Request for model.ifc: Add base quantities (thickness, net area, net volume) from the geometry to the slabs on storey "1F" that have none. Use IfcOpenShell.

First a look at what the model holds.

```python
import ifcopenshell
import ifcopenshell.util.element
import ifcopenshell.util.unit

model = ifcopenshell.open("model.ifc")
print(model.schema)
for unit_type in ("LENGTHUNIT", "AREAUNIT", "VOLUMEUNIT"):
    print(unit_type, ifcopenshell.util.unit.calculate_unit_scale(model, unit_type))
storey = next(s for s in model.by_type("IfcBuildingStorey") if s.Name == "1F")
slabs = [e for e in ifcopenshell.util.element.get_decomposition(storey) if e.is_a("IfcSlab")]
for e in sorted(slabs, key=lambda e: e.id()):
    print(e.id(), e.is_a(), e.Name, list(ifcopenshell.util.element.get_psets(e, qtos_only=True)), sep=" | ")
```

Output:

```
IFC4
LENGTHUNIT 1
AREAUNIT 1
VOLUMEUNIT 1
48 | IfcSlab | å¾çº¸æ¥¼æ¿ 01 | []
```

```python
import ifcopenshell
import ifcopenshell.api.pset
import ifcopenshell.geom
import ifcopenshell.util.element
import ifcopenshell.util.shape
import ifcopenshell.util.unit

model = ifcopenshell.open("model.ifc")
unit_scale = ifcopenshell.util.unit.calculate_unit_scale(model)
area_scale = ifcopenshell.util.unit.calculate_unit_scale(model, "AREAUNIT")
volume_scale = ifcopenshell.util.unit.calculate_unit_scale(model, "VOLUMEUNIT")
settings = ifcopenshell.geom.settings()

storey = next(s for s in model.by_type("IfcBuildingStorey") if s.Name == "1F")
slabs = [e for e in ifcopenshell.util.element.get_decomposition(storey) if e.is_a("IfcSlab")]

for e in sorted(slabs, key=lambda e: e.id()):
    if ifcopenshell.util.element.get_psets(e, qtos_only=True, should_inherit=False):
        continue
    # Geometry comes back in metres, in the element's own axes.
    shape = ifcopenshell.geom.create_shape(settings, e)
    values = {
        "Width": ifcopenshell.util.shape.get_z(shape.geometry) / unit_scale,
        "NetArea": ifcopenshell.util.shape.get_footprint_area(shape.geometry) / area_scale,
        "NetVolume": ifcopenshell.util.shape.get_volume(shape.geometry) / volume_scale,
    }
    qto = ifcopenshell.api.pset.add_qto(model, product=e, name="Qto_SlabBaseQuantities")
    ifcopenshell.api.pset.edit_qto(model, qto=qto, properties=values)
    print(e.id(), {k: round(v, 3) for k, v in values.items()})

model.write("model-out.ifc")
```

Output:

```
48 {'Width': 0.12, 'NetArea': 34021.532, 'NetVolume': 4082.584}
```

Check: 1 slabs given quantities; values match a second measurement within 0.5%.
